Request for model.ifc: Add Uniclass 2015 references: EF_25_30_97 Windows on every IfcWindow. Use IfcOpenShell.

First a look at what the model holds.

```python
import ifcopenshell

model = ifcopenshell.open("model.ifc")
print(model.schema)
print("classifications:", [c.Name for c in model.by_type("IfcClassification")])
for ifc_class in ("IfcDoor", "IfcRoof", "IfcStair", "IfcWall", "IfcWindow"):
    print(ifc_class, len(model.by_type(ifc_class)))
```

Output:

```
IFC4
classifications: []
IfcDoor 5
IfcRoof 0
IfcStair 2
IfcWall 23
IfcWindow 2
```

```python
import ifcopenshell
import ifcopenshell.api.classification

model = ifcopenshell.open("model.ifc")

system = ifcopenshell.api.classification.add_classification(model, classification="Uniclass 2015")

codes = {
    "IfcWindow": ("EF_25_30_97", "Windows"),
}
for ifc_class, (code, name) in codes.items():
    products = model.by_type(ifc_class)
    ifcopenshell.api.classification.add_reference(
        model, products=products, classification=system, identification=code, name=name
    )
    print(code, len(products))

model.write("model-out.ifc")
```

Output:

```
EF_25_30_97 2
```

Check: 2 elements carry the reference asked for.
